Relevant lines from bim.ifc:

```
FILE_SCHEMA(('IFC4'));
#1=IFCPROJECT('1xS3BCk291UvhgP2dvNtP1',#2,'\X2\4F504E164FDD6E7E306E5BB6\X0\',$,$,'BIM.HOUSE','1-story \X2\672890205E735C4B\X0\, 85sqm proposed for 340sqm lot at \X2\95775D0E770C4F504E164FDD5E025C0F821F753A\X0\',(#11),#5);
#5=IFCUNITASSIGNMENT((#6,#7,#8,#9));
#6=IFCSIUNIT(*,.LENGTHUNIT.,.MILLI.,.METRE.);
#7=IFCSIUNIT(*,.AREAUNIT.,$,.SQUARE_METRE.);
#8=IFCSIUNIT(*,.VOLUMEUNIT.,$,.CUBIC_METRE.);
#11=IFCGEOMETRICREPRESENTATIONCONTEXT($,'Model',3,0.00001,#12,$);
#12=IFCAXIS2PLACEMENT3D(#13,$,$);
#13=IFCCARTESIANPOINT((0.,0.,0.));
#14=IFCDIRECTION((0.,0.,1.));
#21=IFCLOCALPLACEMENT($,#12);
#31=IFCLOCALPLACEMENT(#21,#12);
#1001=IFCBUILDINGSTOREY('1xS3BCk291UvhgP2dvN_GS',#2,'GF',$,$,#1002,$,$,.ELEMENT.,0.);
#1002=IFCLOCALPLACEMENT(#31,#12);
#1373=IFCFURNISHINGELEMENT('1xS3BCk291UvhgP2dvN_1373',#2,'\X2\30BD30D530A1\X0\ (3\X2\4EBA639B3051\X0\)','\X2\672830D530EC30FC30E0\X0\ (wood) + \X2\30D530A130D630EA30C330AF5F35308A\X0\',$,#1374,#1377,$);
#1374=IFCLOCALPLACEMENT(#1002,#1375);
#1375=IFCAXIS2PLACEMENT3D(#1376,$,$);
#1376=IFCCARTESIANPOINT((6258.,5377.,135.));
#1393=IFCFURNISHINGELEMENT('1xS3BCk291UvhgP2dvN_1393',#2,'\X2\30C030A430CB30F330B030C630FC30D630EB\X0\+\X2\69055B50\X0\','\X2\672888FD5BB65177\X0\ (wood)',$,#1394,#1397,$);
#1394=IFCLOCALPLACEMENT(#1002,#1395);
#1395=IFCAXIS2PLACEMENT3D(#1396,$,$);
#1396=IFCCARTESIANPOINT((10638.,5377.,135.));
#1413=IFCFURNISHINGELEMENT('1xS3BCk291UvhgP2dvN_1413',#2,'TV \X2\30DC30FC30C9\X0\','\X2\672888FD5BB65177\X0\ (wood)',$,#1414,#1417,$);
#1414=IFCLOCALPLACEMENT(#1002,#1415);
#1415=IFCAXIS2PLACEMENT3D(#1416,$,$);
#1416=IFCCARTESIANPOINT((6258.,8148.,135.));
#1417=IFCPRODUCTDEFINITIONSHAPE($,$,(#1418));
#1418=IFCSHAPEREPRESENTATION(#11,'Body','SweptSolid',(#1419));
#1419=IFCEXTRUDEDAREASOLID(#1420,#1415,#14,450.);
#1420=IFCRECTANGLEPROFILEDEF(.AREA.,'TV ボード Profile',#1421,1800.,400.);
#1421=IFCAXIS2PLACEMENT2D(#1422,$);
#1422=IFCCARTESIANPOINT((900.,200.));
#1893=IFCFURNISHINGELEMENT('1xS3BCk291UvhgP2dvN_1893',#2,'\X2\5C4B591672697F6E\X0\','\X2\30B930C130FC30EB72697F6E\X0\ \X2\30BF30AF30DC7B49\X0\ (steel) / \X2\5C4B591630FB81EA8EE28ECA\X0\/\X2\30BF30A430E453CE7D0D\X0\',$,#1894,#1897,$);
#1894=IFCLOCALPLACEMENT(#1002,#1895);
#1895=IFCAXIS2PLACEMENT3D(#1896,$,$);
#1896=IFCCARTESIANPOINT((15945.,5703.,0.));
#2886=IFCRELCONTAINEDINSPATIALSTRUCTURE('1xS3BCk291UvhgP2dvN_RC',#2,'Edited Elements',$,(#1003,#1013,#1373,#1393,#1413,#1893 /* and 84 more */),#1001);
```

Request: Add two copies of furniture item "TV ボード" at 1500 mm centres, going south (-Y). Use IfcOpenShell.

```python
import numpy as np
import ifcopenshell
import ifcopenshell.api.geometry
import ifcopenshell.api.root
import ifcopenshell.util.element
import ifcopenshell.util.placement

model = ifcopenshell.open("bim.ifc")


def reuse_history(source, copy):
    """copy_class also copies each property set's owner history, people and application; keep the originals."""
    for rel in copy.IsDefinedBy:
        if rel.is_a("IfcRelDefinesByProperties") and (history := rel.RelatingPropertyDefinition.OwnerHistory):
            rel.RelatingPropertyDefinition.OwnerHistory = source.OwnerHistory
            ifcopenshell.util.element.remove_deep2(model, history)


source = model.by_id(1413)
base = ifcopenshell.util.placement.get_local_placement(source.ObjectPlacement)
step = np.array([0.0, -1.0, 0.0]) * 1500.0

for i in range(1, 3):
    copy = ifcopenshell.api.root.copy_class(model, product=source)
    copy.Representation = ifcopenshell.util.element.copy_deep(
        model, source.Representation, exclude=["IfcGeometricRepresentationContext", "IfcRepresentationMap"]
    )
    reuse_history(source, copy)
    matrix = base.copy()
    matrix[:3, 3] += i * step
    print("added at", matrix[:3, 3].round(3) + 0.0)
    ifcopenshell.api.geometry.edit_object_placement(model, product=copy, matrix=matrix, is_si=False)

model.write("bim_updated.ifc")
```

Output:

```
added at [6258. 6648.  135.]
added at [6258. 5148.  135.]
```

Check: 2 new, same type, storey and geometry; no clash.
